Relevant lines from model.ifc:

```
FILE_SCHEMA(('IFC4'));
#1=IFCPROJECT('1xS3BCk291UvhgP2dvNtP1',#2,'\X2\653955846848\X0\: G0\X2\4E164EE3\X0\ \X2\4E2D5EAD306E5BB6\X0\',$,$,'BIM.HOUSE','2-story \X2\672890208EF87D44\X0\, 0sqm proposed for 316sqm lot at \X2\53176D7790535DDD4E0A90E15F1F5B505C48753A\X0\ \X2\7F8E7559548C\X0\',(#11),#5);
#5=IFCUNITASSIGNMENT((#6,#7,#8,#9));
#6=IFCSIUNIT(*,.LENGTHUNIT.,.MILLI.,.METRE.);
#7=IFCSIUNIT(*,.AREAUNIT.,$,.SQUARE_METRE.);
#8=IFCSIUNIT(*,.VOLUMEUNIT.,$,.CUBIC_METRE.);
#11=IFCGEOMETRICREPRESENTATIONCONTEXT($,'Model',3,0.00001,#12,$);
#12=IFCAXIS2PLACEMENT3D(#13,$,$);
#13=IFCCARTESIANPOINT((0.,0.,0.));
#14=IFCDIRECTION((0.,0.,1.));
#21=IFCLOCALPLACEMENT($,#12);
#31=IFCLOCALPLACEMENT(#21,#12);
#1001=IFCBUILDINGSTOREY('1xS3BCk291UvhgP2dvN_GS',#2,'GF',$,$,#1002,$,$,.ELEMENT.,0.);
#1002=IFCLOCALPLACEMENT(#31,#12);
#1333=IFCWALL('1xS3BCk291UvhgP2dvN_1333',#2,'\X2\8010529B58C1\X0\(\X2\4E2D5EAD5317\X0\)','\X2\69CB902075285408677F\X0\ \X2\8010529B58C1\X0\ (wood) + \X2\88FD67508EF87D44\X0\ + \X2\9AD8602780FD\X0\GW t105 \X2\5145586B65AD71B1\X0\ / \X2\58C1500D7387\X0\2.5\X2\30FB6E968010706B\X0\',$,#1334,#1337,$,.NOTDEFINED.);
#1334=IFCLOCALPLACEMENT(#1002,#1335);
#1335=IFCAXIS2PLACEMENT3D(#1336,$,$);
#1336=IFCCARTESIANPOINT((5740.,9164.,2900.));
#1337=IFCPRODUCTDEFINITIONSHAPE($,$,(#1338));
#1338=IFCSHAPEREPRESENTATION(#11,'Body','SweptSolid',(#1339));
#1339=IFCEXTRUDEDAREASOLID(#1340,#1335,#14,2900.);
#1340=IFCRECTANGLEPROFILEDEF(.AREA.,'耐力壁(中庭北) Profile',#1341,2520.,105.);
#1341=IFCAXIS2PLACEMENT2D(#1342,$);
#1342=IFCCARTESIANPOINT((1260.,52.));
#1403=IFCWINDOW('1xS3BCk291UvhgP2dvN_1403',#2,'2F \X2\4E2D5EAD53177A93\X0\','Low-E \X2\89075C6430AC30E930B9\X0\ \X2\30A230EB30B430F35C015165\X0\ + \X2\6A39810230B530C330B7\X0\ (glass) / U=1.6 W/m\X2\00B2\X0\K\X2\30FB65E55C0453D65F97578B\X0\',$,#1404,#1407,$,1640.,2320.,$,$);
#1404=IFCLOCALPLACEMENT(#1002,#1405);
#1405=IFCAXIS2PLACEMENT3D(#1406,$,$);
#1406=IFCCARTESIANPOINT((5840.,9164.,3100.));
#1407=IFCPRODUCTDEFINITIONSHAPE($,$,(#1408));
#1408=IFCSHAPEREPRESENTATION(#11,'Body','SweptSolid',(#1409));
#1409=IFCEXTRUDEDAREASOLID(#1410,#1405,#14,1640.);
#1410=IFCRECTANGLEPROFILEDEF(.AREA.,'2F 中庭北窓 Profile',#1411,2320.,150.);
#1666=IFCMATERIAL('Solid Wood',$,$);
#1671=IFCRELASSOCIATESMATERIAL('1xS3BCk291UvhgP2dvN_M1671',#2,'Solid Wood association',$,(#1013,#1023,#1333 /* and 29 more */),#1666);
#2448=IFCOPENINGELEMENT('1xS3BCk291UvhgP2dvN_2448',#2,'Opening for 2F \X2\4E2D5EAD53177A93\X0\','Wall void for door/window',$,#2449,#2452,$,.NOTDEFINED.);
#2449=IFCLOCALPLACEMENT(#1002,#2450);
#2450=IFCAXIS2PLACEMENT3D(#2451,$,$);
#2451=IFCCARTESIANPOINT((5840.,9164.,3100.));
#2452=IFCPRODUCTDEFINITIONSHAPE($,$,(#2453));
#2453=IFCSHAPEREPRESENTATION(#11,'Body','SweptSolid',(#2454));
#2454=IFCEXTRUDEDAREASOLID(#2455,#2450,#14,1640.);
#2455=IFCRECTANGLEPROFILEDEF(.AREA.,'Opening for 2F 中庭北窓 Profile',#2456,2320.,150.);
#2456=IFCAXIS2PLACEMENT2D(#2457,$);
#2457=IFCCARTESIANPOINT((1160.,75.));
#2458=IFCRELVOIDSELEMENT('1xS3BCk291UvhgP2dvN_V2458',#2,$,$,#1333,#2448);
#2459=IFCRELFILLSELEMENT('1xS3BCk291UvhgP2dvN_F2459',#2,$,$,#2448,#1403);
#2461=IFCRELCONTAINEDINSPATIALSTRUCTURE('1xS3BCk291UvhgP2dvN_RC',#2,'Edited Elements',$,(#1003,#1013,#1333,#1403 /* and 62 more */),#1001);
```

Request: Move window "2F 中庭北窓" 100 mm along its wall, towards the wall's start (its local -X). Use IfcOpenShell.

```python
import ifcopenshell
import ifcopenshell.api.geometry
import ifcopenshell.util.placement

model = ifcopenshell.open("model.ifc")

window = model.by_id(1403)
opening = window.FillsVoids[0].RelatingOpeningElement
wall = opening.VoidsElements[0].RelatingBuildingElement

wall_matrix = ifcopenshell.util.placement.get_local_placement(wall.ObjectPlacement)
shift = wall_matrix[:3, 0] * -100.0
before = ifcopenshell.util.placement.get_local_placement(window.ObjectPlacement)[:3, 3].copy()

# The window is not placed relative to its opening, so move both.
for product in (opening, window):
    matrix = ifcopenshell.util.placement.get_local_placement(product.ObjectPlacement)
    matrix[:3, 3] += shift
    ifcopenshell.api.geometry.edit_object_placement(model, product=product, matrix=matrix, is_si=False)

after = ifcopenshell.util.placement.get_local_placement(window.ObjectPlacement)[:3, 3]
print("window moved by", (after - before).round(3) + 0.0)

model.write("model_rev.ifc")
```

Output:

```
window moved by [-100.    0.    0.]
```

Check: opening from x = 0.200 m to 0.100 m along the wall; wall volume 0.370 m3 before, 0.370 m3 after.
